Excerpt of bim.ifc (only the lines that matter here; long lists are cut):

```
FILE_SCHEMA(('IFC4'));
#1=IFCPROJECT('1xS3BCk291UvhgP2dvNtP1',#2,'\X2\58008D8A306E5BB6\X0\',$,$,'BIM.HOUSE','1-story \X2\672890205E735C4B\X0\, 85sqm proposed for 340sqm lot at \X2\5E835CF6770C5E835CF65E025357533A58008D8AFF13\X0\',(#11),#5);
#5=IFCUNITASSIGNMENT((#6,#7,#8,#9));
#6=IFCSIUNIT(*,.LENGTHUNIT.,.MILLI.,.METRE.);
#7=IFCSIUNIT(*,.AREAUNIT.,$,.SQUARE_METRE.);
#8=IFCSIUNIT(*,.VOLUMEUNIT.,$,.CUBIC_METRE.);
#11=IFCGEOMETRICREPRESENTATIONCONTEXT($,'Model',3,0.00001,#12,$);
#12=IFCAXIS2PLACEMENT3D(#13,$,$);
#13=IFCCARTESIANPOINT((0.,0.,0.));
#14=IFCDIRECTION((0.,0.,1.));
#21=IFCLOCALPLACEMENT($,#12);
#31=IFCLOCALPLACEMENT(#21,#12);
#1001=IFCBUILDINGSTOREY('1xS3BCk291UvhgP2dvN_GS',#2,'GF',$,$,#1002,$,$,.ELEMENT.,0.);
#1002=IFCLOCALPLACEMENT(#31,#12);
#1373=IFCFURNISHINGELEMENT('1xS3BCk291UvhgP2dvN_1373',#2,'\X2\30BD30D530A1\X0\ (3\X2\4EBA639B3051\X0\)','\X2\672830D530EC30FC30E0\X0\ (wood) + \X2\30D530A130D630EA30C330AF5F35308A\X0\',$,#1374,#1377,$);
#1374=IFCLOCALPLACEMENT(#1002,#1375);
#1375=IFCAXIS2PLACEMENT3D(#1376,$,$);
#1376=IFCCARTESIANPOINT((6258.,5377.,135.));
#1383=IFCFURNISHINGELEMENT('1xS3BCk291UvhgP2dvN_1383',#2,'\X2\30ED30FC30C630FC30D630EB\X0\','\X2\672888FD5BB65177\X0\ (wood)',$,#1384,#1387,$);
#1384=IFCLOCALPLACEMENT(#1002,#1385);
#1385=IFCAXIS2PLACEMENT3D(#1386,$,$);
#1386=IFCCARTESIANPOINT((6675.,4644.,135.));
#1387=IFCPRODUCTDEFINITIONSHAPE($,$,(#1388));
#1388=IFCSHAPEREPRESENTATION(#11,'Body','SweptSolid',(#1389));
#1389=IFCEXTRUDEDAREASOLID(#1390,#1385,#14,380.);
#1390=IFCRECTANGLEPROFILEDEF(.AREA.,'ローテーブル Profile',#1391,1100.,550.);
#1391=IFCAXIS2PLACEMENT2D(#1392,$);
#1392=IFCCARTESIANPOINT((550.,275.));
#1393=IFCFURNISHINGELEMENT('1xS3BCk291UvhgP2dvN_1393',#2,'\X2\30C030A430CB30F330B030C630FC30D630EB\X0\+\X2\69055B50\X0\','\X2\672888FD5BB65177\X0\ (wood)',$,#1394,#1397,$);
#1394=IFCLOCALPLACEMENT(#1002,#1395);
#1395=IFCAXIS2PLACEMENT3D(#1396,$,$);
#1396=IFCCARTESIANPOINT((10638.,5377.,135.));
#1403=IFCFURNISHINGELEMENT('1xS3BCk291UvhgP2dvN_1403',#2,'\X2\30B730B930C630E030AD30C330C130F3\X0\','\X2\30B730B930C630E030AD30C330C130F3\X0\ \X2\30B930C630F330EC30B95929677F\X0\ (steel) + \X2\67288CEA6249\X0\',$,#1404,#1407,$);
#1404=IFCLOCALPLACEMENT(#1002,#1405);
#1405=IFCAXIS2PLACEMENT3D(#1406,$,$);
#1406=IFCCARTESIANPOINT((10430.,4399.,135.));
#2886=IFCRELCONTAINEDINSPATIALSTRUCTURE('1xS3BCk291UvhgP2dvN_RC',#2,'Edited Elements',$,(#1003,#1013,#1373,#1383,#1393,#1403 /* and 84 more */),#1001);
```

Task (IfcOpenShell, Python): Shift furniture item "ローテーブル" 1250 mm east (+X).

```python
import ifcopenshell
import ifcopenshell.api.geometry
import ifcopenshell.util.placement
import ifcopenshell.util.unit

model = ifcopenshell.open("bim.ifc")
unit_scale = ifcopenshell.util.unit.calculate_unit_scale(model)

item = model.by_guid("1xS3BCk291UvhgP2dvN_1383")
matrix = ifcopenshell.util.placement.get_local_placement(item.ObjectPlacement)
matrix[0, 3] += 1.25 / unit_scale
ifcopenshell.api.geometry.edit_object_placement(model, product=item, matrix=matrix, is_si=False)

print(ifcopenshell.util.placement.get_local_placement(item.ObjectPlacement).round(3) + 0.0)

model.write("bim_edited.ifc")
```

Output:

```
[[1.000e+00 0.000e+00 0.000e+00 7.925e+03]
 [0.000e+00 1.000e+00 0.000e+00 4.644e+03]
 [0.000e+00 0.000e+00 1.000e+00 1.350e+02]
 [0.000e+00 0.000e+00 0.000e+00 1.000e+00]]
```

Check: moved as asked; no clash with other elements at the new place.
